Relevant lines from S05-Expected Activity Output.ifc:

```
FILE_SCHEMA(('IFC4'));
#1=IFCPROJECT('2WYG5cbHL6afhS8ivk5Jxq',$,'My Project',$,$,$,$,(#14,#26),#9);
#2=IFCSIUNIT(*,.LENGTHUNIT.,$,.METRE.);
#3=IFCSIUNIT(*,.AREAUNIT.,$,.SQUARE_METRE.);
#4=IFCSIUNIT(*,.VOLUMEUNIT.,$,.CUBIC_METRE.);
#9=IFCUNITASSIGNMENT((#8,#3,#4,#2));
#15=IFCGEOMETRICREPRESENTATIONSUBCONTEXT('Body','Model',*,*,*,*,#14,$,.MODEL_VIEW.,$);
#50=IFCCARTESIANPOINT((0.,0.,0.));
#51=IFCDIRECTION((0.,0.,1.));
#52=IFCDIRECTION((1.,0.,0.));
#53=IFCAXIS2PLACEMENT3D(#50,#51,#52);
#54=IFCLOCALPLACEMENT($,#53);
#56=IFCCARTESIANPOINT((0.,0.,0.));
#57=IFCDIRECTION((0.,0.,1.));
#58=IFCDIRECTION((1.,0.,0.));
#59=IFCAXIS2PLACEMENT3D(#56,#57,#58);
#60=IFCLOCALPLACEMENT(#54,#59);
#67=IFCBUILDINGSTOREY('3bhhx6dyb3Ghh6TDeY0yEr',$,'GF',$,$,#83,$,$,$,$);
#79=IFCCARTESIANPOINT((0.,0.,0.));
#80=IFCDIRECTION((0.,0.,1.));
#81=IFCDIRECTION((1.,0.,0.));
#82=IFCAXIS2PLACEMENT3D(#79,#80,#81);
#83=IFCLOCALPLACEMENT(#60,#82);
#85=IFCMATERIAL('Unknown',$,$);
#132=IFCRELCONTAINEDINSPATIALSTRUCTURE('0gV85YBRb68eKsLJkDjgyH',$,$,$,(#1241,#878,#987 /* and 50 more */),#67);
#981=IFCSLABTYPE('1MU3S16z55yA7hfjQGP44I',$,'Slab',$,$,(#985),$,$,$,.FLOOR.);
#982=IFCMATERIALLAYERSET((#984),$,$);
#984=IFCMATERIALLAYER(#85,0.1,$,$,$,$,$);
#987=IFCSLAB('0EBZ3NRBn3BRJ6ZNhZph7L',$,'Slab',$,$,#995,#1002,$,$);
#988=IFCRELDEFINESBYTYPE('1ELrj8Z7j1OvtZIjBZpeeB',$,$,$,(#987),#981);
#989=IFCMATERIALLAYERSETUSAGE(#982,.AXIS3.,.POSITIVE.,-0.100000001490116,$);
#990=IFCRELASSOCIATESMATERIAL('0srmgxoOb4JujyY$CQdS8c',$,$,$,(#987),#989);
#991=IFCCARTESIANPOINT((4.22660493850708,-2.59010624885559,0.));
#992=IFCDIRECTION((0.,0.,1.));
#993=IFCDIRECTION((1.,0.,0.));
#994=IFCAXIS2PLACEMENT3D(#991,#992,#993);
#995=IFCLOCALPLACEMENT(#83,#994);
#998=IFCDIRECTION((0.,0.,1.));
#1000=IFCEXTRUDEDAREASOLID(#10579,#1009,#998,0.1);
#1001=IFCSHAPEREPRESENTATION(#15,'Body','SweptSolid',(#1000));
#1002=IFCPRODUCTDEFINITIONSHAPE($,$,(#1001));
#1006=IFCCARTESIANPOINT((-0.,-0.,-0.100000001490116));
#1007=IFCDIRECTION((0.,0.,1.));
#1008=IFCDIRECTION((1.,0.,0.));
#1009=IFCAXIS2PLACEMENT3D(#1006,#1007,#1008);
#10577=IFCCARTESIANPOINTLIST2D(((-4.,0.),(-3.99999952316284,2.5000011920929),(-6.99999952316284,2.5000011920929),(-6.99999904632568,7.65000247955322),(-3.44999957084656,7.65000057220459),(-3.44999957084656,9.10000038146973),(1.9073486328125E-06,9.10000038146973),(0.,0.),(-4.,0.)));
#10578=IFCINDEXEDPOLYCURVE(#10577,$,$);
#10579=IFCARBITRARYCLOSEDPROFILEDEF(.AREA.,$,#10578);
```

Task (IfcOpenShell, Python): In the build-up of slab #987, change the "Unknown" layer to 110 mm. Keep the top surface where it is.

```python
import ifcopenshell
import ifcopenshell.util.element
import ifcopenshell.util.representation

model = ifcopenshell.open("S05-Expected Activity Output.ifc")

layer_set = model.by_id(982)
layer = next(l for l in layer_set.MaterialLayers if l.Material and l.Material.Name == "Unknown")
change = 0.11 - layer.LayerThickness
layer.LayerThickness += change

# Geometry does not follow the layer set by itself.
slabs = [e for e in ifcopenshell.util.element.get_elements_by_material(model, layer_set) if e.is_a("IfcSlab")]
for slab in sorted(slabs, key=lambda e: e.id()):
    body = ifcopenshell.util.representation.get_representation(slab, "Model", "Body")
    solid = body.Items[0]
    old_depth = solid.Depth
    solid.Depth += change
    # Extruded upwards: lower the start of the extrusion so the top stays.
    x, y, z = solid.Position.Location.Coordinates
    solid.Position.Location = model.createIfcCartesianPoint((x, y, z - change))
    print(slab.id(), f"{old_depth:g} -> {solid.Depth:g}")

# The layers are counted up from the underside, which has moved.
for usage in {ifcopenshell.util.element.get_material(slab) for slab in slabs}:
    usage.OffsetFromReferenceLine -= change

model.write("S05-Expected Activity Output_edited.ifc")
```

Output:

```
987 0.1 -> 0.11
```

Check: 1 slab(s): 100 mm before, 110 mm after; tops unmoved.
